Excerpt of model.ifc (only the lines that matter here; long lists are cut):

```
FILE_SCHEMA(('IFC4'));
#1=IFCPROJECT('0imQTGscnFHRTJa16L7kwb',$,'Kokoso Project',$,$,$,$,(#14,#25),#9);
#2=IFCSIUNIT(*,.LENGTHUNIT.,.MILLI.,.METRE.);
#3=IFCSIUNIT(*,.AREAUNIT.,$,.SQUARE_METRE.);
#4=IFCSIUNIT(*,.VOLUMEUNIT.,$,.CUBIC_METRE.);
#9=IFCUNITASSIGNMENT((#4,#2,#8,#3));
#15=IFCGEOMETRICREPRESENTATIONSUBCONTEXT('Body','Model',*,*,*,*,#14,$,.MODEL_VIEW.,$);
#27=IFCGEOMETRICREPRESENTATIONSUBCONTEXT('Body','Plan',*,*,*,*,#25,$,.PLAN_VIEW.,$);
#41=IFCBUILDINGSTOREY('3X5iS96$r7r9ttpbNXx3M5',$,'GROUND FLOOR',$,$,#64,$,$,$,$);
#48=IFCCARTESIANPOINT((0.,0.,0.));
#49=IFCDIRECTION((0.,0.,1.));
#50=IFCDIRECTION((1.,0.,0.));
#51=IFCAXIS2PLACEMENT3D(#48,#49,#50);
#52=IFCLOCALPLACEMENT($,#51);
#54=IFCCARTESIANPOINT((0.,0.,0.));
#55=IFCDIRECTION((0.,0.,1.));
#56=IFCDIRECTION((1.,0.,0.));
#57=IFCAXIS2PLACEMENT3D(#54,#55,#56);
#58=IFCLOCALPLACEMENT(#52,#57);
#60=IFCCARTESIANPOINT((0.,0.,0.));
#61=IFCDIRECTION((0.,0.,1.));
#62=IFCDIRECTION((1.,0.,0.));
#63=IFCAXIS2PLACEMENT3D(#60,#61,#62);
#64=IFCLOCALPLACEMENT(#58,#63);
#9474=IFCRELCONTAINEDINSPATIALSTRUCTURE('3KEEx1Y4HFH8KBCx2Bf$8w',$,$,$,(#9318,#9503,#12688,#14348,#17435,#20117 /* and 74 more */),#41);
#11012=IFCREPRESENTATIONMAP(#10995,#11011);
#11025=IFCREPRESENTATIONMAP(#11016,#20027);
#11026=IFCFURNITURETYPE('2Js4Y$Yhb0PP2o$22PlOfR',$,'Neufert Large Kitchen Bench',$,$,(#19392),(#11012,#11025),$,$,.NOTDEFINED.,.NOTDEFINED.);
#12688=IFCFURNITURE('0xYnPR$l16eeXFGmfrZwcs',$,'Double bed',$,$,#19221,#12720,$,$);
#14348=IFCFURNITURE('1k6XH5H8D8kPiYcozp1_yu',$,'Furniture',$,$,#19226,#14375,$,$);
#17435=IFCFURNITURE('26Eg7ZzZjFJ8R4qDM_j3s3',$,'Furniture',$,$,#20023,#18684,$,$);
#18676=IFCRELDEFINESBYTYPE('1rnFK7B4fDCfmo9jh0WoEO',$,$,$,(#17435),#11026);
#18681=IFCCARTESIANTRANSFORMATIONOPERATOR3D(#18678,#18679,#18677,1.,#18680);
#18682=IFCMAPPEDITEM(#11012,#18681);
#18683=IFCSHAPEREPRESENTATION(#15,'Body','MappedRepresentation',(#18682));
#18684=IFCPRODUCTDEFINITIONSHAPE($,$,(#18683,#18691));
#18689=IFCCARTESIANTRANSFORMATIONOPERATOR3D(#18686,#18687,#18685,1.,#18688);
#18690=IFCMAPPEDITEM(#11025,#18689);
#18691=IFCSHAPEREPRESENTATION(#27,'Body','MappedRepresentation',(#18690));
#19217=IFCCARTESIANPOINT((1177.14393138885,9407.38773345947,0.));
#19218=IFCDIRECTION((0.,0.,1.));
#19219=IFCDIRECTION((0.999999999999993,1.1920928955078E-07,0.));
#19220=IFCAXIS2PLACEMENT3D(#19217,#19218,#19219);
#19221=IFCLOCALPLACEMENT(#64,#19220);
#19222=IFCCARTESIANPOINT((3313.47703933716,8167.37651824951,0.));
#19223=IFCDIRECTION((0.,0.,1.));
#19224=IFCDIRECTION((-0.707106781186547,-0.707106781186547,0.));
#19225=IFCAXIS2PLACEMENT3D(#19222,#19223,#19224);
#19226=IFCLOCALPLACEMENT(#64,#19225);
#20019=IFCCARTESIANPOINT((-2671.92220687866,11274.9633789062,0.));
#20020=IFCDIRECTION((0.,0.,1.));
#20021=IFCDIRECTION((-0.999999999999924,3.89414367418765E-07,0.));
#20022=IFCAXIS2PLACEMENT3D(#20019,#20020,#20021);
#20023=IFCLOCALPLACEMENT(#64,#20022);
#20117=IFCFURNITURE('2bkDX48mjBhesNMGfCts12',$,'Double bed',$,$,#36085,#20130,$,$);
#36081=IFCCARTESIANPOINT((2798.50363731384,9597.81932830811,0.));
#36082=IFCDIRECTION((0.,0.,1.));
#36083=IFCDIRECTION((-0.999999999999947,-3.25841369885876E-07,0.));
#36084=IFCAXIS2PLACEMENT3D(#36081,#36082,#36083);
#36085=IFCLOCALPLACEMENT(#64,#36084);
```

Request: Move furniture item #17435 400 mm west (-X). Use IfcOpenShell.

```python
import ifcopenshell
import ifcopenshell.api.geometry
import ifcopenshell.util.placement

model = ifcopenshell.open("model.ifc")

item = model.by_guid("26Eg7ZzZjFJ8R4qDM_j3s3")
matrix = ifcopenshell.util.placement.get_local_placement(item.ObjectPlacement)
matrix[0, 3] -= 400.0
ifcopenshell.api.geometry.edit_object_placement(model, product=item, matrix=matrix, is_si=False)

print(ifcopenshell.util.placement.get_local_placement(item.ObjectPlacement).round(3) + 0.0)

model.write("model_v2.ifc")
```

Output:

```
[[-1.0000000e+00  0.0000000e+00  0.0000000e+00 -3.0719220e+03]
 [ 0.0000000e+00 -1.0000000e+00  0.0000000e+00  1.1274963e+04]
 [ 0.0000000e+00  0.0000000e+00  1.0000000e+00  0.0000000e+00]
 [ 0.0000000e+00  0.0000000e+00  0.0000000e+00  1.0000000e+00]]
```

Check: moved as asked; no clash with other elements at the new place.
